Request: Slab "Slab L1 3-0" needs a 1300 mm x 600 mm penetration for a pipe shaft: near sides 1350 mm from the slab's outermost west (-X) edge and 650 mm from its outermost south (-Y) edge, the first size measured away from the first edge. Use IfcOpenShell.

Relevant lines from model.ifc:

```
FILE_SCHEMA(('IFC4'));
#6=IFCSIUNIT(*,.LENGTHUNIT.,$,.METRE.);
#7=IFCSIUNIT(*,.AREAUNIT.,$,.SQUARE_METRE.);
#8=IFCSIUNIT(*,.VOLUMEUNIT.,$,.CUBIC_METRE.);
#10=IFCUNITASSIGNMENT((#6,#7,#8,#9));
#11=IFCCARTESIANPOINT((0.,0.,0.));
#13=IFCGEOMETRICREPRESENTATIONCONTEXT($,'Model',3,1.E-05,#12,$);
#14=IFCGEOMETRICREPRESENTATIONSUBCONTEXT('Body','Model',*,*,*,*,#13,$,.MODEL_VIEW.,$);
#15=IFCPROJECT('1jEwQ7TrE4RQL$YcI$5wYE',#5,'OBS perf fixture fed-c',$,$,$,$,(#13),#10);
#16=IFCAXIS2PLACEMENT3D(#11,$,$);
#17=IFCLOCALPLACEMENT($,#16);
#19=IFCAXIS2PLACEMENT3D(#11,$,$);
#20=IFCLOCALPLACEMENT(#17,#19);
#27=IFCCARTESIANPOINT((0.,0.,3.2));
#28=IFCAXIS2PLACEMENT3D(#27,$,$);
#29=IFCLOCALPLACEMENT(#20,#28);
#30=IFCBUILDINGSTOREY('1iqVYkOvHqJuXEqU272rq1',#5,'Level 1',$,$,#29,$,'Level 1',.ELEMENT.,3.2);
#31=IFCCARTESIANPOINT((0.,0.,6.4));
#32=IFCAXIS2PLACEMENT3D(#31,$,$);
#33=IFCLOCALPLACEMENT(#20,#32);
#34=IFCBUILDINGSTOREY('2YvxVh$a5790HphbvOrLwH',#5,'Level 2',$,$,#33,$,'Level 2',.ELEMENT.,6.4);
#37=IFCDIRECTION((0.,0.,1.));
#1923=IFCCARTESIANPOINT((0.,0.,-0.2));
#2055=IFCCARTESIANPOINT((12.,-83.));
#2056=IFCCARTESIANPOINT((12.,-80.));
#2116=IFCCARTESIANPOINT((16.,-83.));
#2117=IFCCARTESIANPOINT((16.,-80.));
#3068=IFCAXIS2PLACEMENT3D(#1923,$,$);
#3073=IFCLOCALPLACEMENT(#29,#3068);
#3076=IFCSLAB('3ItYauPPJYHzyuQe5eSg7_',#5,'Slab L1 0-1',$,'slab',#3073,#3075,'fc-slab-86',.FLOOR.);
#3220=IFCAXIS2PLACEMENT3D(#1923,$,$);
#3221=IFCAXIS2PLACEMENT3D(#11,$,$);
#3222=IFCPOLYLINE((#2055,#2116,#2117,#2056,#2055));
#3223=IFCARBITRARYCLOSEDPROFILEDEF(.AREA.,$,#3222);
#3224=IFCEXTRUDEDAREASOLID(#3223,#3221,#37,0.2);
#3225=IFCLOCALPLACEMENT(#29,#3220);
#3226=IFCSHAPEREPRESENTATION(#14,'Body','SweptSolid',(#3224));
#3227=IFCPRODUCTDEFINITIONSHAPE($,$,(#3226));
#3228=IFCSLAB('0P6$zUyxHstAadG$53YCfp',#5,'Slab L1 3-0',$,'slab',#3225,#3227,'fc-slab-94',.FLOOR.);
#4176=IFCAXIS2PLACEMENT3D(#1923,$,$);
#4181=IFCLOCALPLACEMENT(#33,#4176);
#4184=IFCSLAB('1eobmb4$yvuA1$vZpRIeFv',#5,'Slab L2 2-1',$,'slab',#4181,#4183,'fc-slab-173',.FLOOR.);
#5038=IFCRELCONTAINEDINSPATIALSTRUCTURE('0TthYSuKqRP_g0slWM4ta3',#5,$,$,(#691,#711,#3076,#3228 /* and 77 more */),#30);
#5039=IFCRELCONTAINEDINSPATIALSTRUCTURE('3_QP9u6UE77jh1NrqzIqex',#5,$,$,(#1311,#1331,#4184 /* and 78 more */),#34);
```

```python
import numpy as np
import ifcopenshell
import ifcopenshell.api.feature
import ifcopenshell.api.geometry
import ifcopenshell.api.root
import ifcopenshell.geom
import ifcopenshell.util.placement
import ifcopenshell.util.representation
import ifcopenshell.util.shape
import ifcopenshell.util.unit

model = ifcopenshell.open("model.ifc")
unit_scale = ifcopenshell.util.unit.calculate_unit_scale(model)
settings = ifcopenshell.geom.settings()


def volume(element):
    """Net volume in cubic metres, openings subtracted."""
    shape = ifcopenshell.geom.create_shape(settings, element)
    return ifcopenshell.util.shape.get_volume(shape.geometry)


slab = model.by_guid("0P6$zUyxHstAadG$53YCfp")
before = volume(slab)

# Extent in the slab's own axes, in metres. The edges named are its -X and -Y sides.
slab_shape = ifcopenshell.geom.create_shape(settings, slab)
vertices = ifcopenshell.util.shape.get_vertices(slab_shape.geometry)
x_min, y_min, bottom = vertices.min(axis=0)
top = vertices[:, 2].max()

opening = ifcopenshell.api.root.create_entity(model, ifc_class="IfcOpeningElement", name="Pipe shaft opening", predefined_type="OPENING")
context = ifcopenshell.util.representation.get_context(model, "Model", "Body", "MODEL_VIEW")
width, depth = 1.3, 0.6
outline = [(0.0, 0.0), (width, 0.0), (width, depth), (0.0, depth), (0.0, 0.0)]
# Overshoot both faces by 50 mm so the cut is clean.
shape = ifcopenshell.api.geometry.add_slab_representation(
    model, context=context, depth=top - bottom + 0.1, polyline=outline
)
ifcopenshell.api.geometry.assign_representation(model, product=opening, representation=shape)

matrix = ifcopenshell.util.placement.get_local_placement(slab.ObjectPlacement)
matrix[:, 3] = matrix @ np.append(np.array([x_min + 1.35, y_min + 0.65, bottom - 0.05]) / unit_scale, 1.0)
ifcopenshell.api.geometry.edit_object_placement(model, product=opening, matrix=matrix, is_si=False)
ifcopenshell.api.feature.add_feature(model, feature=opening, element=slab)

after = volume(slab)

print(f"slab volume {before:.3f} -> {after:.3f} m3")

model.write("model-out.ifc")
```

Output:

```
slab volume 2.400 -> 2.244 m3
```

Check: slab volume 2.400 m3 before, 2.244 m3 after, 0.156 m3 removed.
